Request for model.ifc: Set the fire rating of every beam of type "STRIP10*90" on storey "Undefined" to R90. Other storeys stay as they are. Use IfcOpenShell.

First a look at what the model holds.

```python
import ifcopenshell
import ifcopenshell.util.element

model = ifcopenshell.open("model.ifc")
print(model.schema)
storey = next(s for s in model.by_type("IfcBuildingStorey") if s.Name == "Undefined")
beams = [e for e in ifcopenshell.util.element.get_decomposition(storey) if e.is_a("IfcBeam")]
seen = {}
for e in beams:
    element_type = ifcopenshell.util.element.get_type(e)
    key = (element_type.Name if element_type != e and element_type else None, ifcopenshell.util.element.get_pset(e, "Pset_BeamCommon", "FireRating"))
    seen[key] = seen.get(key, 0) + 1
for (name, value), count in sorted(seen.items(), key=str):
    print(count, "x", name, "|", value)
```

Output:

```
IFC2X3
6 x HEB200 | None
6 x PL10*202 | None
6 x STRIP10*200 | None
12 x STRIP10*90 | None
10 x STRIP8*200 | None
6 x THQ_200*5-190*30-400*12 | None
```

```python
import ifcopenshell
import ifcopenshell.api.pset
import ifcopenshell.util.element

model = ifcopenshell.open("model.ifc")

storey = next(s for s in model.by_type("IfcBuildingStorey") if s.Name == "Undefined")
beams = [e for e in ifcopenshell.util.element.get_decomposition(storey) if e.is_a("IfcBeam")]

count = 0
for e in beams:
    element_type = ifcopenshell.util.element.get_type(e)
    if element_type in (None, e) or element_type.Name != "STRIP10*90":
        continue
    # add_pset returns the element's existing set when there is one.
    pset = ifcopenshell.api.pset.add_pset(model, product=e, name="Pset_BeamCommon")
    ifcopenshell.api.pset.edit_pset(model, pset=pset, properties={"FireRating": "R90"})
    count += 1

print(count, "beams updated")

model.write("model_rev.ifc")
```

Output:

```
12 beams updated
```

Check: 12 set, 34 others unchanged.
